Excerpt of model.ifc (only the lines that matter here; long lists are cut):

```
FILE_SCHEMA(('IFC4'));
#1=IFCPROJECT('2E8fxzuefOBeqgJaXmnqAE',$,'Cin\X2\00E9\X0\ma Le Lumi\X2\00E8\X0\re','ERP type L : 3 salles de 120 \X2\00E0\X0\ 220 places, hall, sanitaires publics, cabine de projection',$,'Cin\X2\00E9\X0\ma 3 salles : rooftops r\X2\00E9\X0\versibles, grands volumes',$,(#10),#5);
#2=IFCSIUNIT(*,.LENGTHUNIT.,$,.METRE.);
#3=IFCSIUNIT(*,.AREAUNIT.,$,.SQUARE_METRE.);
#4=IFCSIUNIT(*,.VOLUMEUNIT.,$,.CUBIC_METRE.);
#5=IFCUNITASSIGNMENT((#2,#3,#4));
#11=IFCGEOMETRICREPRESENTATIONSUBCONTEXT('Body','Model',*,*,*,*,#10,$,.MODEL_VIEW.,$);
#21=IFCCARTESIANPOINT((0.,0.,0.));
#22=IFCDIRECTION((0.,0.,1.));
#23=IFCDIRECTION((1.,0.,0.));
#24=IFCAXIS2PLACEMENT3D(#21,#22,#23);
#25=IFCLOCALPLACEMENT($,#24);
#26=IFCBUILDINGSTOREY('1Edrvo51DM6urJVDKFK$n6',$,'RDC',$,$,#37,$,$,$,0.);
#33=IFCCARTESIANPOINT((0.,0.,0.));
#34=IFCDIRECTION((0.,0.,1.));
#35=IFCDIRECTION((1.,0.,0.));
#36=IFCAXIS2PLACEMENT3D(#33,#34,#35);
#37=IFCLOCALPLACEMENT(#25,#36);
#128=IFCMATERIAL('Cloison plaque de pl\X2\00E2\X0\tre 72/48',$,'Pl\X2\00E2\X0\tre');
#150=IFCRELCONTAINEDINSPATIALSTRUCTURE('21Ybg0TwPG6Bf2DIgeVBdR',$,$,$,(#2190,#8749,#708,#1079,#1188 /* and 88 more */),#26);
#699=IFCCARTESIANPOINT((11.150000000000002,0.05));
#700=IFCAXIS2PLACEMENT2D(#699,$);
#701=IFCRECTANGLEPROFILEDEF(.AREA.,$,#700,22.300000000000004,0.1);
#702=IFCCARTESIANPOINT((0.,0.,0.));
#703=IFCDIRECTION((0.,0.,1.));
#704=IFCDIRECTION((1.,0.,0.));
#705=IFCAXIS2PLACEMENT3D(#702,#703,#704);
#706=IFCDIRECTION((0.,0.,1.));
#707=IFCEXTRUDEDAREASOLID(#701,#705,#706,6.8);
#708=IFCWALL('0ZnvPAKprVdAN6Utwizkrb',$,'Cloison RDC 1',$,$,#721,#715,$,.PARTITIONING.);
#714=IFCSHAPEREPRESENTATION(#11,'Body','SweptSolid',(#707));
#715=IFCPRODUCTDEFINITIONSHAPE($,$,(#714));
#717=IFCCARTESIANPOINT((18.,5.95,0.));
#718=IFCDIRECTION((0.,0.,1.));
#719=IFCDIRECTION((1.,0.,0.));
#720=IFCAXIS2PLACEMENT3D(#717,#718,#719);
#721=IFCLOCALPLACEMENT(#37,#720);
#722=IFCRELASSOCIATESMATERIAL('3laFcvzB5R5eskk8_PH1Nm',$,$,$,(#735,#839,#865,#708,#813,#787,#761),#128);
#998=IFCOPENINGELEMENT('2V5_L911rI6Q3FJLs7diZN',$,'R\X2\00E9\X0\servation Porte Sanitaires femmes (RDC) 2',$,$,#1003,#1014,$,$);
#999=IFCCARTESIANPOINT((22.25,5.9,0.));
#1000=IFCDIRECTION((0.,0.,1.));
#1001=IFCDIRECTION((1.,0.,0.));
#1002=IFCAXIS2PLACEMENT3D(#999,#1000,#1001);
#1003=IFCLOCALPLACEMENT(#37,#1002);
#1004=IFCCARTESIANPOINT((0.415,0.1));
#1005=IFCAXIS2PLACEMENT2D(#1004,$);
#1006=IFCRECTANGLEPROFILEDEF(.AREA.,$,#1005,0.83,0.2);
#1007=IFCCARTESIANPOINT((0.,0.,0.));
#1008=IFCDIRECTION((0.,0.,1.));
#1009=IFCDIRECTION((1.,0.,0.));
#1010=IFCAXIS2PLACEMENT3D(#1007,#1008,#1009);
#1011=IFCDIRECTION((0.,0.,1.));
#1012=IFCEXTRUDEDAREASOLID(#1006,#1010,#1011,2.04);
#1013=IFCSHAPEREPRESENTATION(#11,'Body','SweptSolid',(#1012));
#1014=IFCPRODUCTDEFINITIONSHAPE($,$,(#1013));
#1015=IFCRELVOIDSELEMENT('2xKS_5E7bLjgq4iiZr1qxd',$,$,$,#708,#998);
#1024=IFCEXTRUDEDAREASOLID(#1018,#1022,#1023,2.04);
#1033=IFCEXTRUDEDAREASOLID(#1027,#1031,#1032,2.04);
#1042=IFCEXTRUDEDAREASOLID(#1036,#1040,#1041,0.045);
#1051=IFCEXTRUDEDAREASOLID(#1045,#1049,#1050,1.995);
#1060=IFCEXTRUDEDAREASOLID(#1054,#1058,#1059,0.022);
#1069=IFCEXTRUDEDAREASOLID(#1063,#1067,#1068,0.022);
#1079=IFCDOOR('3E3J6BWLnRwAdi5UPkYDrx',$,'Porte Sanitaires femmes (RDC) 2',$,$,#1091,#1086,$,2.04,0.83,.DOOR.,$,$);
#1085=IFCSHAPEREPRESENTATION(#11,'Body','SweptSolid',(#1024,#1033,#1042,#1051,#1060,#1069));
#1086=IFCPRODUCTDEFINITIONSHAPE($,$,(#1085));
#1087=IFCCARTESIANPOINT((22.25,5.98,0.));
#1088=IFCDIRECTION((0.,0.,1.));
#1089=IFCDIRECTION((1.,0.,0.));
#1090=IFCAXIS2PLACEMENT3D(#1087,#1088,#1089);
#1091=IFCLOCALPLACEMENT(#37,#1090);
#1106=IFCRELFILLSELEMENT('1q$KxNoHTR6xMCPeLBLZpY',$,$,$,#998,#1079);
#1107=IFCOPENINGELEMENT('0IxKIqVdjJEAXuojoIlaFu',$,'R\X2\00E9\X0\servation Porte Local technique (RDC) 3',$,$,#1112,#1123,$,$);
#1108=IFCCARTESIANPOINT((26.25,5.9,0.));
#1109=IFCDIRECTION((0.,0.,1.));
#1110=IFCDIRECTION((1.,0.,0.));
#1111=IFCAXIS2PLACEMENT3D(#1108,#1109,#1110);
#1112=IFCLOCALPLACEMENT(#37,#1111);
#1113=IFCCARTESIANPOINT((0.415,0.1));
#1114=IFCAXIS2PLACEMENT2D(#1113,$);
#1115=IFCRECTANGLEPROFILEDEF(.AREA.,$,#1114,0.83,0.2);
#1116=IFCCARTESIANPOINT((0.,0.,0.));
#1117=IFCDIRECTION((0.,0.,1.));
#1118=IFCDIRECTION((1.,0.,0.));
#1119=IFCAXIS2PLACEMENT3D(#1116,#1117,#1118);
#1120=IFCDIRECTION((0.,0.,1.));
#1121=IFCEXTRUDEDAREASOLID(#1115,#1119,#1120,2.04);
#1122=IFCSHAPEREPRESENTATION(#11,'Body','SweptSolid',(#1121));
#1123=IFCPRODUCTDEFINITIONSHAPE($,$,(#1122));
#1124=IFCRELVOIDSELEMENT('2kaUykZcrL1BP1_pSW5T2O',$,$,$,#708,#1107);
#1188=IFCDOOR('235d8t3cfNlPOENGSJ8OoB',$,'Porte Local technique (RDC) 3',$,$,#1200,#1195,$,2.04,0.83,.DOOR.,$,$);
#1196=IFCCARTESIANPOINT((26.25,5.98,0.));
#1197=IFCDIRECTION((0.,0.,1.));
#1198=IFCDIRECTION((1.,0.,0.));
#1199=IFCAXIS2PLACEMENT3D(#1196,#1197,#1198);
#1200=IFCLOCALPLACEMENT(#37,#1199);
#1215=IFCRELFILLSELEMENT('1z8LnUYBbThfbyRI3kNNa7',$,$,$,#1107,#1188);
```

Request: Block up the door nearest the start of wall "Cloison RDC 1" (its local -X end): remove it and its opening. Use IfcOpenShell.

```python
import ifcopenshell
import ifcopenshell.api.feature
import ifcopenshell.api.root
import ifcopenshell.geom
import ifcopenshell.util.shape

model = ifcopenshell.open("model.ifc")
settings = ifcopenshell.geom.settings()


def volume(element):
    """Net volume in cubic metres, openings subtracted."""
    shape = ifcopenshell.geom.create_shape(settings, element)
    return ifcopenshell.util.shape.get_volume(shape.geometry)


door = model.by_guid("3E3J6BWLnRwAdi5UPkYDrx")
opening = door.FillsVoids[0].RelatingOpeningElement
wall = opening.VoidsElements[0].RelatingBuildingElement
before = volume(wall)

ifcopenshell.api.root.remove_product(model, product=door)
ifcopenshell.api.feature.remove_feature(model, feature=opening)

after = volume(wall)

print(f"wall volume {before:.3f} -> {after:.3f} m3")

model.write("model-out.ifc")
```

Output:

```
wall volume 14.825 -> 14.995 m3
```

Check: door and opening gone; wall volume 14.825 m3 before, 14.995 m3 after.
